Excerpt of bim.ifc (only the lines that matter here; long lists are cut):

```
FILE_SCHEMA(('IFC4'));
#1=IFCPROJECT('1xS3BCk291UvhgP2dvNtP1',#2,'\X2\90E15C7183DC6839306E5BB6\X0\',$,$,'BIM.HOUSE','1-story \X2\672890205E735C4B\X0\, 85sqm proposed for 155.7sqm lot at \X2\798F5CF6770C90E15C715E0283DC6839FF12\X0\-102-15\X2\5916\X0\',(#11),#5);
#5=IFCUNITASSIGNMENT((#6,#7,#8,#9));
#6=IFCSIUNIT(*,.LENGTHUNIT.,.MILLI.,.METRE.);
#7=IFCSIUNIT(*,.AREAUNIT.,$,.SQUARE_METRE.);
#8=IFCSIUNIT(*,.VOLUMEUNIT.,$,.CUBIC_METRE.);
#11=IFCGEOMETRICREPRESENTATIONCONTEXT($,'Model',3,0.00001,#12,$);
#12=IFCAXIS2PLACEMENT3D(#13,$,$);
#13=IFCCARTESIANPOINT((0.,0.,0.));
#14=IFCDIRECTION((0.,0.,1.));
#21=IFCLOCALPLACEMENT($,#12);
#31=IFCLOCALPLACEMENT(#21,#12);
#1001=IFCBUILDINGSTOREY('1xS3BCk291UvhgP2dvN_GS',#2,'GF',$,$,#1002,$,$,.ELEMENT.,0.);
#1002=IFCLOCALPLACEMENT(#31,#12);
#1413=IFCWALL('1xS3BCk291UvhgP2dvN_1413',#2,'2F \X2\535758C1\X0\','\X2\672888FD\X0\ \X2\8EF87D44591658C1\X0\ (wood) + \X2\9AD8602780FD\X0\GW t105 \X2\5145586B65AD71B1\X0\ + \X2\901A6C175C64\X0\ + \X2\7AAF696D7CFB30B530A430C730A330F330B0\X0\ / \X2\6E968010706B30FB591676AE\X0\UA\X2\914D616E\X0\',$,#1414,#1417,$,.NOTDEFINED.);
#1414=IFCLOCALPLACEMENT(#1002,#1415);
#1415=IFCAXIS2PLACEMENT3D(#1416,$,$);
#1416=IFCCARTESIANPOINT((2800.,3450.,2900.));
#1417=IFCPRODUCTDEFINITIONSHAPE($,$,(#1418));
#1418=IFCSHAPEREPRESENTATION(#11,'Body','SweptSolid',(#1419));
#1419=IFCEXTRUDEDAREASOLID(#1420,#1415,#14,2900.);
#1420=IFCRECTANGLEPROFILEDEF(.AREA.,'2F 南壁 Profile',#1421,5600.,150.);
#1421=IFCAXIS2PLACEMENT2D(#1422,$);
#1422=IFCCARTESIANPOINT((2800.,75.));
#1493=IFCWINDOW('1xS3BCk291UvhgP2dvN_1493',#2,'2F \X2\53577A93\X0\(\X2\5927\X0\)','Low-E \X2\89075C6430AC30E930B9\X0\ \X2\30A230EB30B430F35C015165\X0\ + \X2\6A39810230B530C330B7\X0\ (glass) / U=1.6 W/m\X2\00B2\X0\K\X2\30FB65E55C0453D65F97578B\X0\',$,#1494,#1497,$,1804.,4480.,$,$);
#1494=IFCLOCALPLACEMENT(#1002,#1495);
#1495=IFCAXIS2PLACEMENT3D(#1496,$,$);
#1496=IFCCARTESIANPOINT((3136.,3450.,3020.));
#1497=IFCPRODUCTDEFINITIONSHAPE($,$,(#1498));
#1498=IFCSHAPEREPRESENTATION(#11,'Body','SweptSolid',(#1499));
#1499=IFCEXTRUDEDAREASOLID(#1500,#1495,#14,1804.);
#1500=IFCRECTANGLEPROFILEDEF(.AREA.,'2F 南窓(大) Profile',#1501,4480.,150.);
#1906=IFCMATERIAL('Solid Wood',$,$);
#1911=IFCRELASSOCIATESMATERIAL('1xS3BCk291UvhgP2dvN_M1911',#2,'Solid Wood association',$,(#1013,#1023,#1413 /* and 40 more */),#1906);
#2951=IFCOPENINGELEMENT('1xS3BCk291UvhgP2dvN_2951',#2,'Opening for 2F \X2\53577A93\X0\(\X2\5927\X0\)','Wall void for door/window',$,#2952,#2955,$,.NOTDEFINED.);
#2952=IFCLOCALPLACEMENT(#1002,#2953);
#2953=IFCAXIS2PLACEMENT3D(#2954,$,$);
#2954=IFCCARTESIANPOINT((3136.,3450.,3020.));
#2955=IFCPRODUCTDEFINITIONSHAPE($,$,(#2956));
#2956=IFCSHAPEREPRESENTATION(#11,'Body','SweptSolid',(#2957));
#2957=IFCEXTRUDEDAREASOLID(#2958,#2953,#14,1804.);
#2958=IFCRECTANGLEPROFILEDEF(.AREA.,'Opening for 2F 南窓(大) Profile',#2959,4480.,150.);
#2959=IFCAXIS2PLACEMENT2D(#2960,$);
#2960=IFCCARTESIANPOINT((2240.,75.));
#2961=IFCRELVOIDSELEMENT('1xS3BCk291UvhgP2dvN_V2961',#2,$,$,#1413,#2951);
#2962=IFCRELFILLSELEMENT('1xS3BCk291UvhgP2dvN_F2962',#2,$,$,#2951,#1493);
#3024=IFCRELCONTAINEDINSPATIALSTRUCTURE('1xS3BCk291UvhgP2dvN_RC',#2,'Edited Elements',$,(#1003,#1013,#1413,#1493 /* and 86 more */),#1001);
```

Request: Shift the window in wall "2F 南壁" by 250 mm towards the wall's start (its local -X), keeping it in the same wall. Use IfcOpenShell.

```python
import ifcopenshell
import ifcopenshell.api.geometry
import ifcopenshell.util.placement
import ifcopenshell.util.unit

model = ifcopenshell.open("bim.ifc")
unit_scale = ifcopenshell.util.unit.calculate_unit_scale(model)

window = model.by_guid("1xS3BCk291UvhgP2dvN_1493")
opening = window.FillsVoids[0].RelatingOpeningElement
wall = opening.VoidsElements[0].RelatingBuildingElement

wall_matrix = ifcopenshell.util.placement.get_local_placement(wall.ObjectPlacement)
shift = wall_matrix[:3, 0] * -0.25 / unit_scale
before = ifcopenshell.util.placement.get_local_placement(window.ObjectPlacement)[:3, 3].copy()

# The window is not placed relative to its opening, so move both.
for product in (opening, window):
    matrix = ifcopenshell.util.placement.get_local_placement(product.ObjectPlacement)
    matrix[:3, 3] += shift
    ifcopenshell.api.geometry.edit_object_placement(model, product=product, matrix=matrix, is_si=False)

after = ifcopenshell.util.placement.get_local_placement(window.ObjectPlacement)[:3, 3]
print("window moved by", (after - before).round(3) + 0.0)

model.write("bim-out.ifc")
```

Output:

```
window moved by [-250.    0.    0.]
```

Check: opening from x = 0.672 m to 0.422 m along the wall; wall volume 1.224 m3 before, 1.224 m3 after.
